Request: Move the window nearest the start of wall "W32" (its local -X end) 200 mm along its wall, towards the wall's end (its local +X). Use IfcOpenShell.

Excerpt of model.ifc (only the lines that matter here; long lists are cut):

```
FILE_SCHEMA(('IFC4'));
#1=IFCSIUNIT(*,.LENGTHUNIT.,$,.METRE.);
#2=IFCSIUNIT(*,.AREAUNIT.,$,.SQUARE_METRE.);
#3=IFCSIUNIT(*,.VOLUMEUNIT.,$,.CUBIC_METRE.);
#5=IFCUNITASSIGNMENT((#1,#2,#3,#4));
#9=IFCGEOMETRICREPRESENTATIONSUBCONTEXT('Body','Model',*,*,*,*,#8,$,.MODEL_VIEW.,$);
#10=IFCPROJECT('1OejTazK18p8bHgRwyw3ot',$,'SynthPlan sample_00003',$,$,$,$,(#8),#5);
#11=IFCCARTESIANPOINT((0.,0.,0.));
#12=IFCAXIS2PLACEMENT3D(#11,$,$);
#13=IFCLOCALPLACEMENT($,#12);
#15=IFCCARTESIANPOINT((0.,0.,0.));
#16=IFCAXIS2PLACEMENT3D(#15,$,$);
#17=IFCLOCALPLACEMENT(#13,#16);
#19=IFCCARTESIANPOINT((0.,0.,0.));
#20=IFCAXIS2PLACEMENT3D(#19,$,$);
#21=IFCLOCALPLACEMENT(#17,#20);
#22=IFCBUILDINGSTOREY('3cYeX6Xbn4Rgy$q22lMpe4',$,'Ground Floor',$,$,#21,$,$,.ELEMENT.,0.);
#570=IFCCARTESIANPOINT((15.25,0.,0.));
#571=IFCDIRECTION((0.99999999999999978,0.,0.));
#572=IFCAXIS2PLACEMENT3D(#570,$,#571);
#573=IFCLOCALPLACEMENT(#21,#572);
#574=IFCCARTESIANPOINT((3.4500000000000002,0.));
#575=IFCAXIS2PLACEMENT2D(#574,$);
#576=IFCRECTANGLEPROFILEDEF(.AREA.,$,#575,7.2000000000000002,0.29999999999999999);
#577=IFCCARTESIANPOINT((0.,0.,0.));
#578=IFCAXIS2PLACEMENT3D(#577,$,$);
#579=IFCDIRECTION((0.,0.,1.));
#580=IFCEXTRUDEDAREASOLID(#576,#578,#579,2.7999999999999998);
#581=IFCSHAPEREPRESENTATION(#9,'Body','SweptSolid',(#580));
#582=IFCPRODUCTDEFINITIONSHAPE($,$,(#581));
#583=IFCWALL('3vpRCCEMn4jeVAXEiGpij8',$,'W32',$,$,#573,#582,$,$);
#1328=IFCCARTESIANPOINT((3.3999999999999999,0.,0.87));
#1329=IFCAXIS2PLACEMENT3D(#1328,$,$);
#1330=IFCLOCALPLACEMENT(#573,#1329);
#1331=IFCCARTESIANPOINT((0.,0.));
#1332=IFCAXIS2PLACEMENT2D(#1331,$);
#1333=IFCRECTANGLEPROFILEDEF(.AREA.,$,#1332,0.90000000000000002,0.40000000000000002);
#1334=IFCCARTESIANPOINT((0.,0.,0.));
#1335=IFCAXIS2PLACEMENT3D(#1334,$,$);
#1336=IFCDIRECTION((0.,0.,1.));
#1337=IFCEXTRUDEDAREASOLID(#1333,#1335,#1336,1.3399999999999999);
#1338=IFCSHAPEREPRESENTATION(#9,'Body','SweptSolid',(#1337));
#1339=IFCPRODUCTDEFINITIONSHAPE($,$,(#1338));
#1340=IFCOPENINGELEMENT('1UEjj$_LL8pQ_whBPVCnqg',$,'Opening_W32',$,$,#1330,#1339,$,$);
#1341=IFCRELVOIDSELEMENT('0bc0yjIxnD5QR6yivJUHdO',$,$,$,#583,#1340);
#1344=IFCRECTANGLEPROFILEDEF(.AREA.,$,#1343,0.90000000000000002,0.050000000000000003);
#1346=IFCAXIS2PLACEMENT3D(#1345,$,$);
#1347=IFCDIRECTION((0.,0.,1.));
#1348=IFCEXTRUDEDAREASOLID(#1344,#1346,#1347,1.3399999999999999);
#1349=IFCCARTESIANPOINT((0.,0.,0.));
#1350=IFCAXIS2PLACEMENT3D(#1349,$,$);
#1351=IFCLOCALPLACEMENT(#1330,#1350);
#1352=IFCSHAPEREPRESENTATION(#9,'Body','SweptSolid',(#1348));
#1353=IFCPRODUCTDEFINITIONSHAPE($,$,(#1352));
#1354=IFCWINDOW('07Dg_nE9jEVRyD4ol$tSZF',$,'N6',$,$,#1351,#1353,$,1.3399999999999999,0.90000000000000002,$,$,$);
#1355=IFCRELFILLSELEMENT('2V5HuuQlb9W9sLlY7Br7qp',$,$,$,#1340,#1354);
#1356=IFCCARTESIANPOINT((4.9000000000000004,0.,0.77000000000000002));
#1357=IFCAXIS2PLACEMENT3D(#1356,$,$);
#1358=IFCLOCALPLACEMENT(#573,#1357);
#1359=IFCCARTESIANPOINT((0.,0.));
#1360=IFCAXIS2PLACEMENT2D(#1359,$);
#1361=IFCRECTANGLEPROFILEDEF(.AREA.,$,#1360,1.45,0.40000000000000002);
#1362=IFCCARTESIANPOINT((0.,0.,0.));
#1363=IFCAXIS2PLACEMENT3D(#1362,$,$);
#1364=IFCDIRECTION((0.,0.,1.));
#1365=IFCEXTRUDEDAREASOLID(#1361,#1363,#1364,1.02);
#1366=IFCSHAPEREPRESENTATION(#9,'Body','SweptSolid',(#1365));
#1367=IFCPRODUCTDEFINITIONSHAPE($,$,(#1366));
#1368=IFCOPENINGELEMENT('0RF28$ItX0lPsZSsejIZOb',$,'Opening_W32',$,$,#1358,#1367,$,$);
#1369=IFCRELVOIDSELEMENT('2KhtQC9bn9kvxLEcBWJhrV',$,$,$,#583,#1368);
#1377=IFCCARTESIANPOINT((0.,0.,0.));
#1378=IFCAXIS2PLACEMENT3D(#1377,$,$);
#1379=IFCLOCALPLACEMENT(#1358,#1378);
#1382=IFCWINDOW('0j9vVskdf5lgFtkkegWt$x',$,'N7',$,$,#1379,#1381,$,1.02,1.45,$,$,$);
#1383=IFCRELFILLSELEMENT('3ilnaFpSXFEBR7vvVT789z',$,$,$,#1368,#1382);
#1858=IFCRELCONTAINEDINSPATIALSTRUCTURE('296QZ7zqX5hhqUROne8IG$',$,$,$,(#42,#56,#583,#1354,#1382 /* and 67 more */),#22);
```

```python
import ifcopenshell
import ifcopenshell.api.geometry
import ifcopenshell.util.placement
import ifcopenshell.util.unit

model = ifcopenshell.open("model.ifc")
unit_scale = ifcopenshell.util.unit.calculate_unit_scale(model)

window = model.by_guid("07Dg_nE9jEVRyD4ol$tSZF")
opening = window.FillsVoids[0].RelatingOpeningElement
wall = opening.VoidsElements[0].RelatingBuildingElement

wall_matrix = ifcopenshell.util.placement.get_local_placement(wall.ObjectPlacement)
shift = wall_matrix[:3, 0] * 0.2 / unit_scale
before = ifcopenshell.util.placement.get_local_placement(window.ObjectPlacement)[:3, 3].copy()

# The window is placed relative to its opening, so it follows when the opening moves.
matrix = ifcopenshell.util.placement.get_local_placement(opening.ObjectPlacement)
matrix[:3, 3] += shift
ifcopenshell.api.geometry.edit_object_placement(
    model, product=opening, matrix=matrix, is_si=False, should_transform_children=True
)

after = ifcopenshell.util.placement.get_local_placement(window.ObjectPlacement)[:3, 3]
print("window moved by", (after - before).round(3) + 0.0)

model.write("model_rev.ifc")
```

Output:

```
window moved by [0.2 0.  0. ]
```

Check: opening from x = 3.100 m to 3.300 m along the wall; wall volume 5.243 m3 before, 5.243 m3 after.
